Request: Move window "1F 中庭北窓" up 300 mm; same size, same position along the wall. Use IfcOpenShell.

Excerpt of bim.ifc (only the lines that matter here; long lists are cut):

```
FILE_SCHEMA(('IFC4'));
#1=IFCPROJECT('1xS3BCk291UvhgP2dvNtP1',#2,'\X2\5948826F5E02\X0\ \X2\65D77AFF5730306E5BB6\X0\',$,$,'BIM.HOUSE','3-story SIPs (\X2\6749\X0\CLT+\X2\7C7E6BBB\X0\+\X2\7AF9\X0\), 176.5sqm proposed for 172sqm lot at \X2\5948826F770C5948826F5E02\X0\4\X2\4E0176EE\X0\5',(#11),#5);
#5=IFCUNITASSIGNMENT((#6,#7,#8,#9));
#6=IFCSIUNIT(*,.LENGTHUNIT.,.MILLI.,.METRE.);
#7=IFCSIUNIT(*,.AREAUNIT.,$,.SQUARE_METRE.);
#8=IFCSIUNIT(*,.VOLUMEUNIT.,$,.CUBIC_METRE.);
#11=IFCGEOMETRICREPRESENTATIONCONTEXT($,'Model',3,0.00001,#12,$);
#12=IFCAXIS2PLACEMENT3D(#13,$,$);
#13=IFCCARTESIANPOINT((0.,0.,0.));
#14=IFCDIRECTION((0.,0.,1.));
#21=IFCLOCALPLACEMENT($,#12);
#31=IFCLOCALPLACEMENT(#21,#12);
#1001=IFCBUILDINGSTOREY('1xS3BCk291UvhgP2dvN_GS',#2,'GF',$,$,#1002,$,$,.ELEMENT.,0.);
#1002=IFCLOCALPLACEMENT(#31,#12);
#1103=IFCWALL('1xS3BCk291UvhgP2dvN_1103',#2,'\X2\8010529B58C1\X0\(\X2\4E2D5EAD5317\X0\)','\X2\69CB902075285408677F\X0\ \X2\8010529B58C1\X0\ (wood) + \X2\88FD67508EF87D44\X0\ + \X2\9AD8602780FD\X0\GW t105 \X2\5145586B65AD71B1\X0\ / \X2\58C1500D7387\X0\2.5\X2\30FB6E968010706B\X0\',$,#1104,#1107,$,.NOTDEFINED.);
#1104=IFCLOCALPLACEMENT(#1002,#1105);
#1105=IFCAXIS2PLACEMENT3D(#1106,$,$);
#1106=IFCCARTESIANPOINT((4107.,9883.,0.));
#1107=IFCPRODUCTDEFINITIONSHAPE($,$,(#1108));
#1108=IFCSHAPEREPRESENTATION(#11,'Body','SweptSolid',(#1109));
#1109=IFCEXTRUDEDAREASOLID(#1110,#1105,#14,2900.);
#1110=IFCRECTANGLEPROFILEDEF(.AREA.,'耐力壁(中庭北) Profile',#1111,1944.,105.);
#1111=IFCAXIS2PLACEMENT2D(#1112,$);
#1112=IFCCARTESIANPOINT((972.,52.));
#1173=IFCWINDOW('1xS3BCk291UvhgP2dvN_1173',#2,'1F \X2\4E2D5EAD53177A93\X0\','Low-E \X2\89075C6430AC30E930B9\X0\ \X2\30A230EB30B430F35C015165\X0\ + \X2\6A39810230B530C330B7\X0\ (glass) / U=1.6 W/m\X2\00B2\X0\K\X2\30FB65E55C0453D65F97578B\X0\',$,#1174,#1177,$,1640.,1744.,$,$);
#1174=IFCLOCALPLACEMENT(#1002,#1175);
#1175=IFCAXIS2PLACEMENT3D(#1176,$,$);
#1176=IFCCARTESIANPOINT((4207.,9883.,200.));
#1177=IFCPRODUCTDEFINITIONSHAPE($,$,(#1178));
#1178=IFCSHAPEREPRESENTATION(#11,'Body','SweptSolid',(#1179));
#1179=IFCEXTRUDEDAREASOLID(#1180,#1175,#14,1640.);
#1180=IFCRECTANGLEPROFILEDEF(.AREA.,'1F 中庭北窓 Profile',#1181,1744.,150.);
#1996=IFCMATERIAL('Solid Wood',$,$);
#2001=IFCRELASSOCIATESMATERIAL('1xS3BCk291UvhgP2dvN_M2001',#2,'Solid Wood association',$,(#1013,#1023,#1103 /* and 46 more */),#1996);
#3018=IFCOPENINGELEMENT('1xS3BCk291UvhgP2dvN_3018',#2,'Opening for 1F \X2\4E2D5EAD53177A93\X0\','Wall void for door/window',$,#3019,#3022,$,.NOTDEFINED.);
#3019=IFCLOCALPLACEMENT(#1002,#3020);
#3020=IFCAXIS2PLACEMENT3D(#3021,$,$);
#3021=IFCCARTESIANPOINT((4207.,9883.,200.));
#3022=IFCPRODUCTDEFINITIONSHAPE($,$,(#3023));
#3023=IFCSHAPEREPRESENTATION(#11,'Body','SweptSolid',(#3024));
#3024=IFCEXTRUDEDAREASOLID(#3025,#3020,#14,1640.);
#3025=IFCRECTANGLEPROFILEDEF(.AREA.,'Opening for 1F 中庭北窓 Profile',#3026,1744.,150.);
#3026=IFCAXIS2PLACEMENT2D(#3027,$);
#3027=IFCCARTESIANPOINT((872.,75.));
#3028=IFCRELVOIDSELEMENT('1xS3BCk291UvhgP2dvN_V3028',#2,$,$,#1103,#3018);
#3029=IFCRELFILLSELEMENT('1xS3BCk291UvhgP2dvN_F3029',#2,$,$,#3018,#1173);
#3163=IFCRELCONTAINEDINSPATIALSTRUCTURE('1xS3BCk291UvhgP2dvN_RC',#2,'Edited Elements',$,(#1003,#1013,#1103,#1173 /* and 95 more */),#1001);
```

```python
import numpy as np
import ifcopenshell
import ifcopenshell.api.geometry
import ifcopenshell.util.placement
import ifcopenshell.util.unit

model = ifcopenshell.open("bim.ifc")
unit_scale = ifcopenshell.util.unit.calculate_unit_scale(model)

window = model.by_id(1173)
opening = window.FillsVoids[0].RelatingOpeningElement
dz = 0.3 / unit_scale

shift = np.array([0.0, 0.0, dz])
# The window is not placed relative to its opening, so move both.
for product in (opening, window):
    matrix = ifcopenshell.util.placement.get_local_placement(product.ObjectPlacement)
    matrix[:3, 3] += shift
    ifcopenshell.api.geometry.edit_object_placement(model, product=product, matrix=matrix, is_si=False)

print(f"moved by {dz * unit_scale:+.3f} m")

model.write("bim_updated.ifc")
```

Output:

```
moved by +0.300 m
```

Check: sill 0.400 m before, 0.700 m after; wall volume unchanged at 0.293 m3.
